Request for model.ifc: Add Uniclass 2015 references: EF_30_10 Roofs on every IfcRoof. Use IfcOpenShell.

First a look at what the model holds.

```python
import ifcopenshell

model = ifcopenshell.open("model.ifc")
print(model.schema)
print("classifications:", [c.Name for c in model.by_type("IfcClassification")])
for ifc_class in ("IfcDoor", "IfcRoof", "IfcStair", "IfcWall", "IfcWindow"):
    print(ifc_class, len(model.by_type(ifc_class)))
```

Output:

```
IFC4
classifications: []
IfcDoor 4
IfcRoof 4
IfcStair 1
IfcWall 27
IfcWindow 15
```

```python
import ifcopenshell
import ifcopenshell.api.classification

model = ifcopenshell.open("model.ifc")

system = ifcopenshell.api.classification.add_classification(model, classification="Uniclass 2015")

codes = {
    "IfcRoof": ("EF_30_10", "Roofs"),
}
for ifc_class, (code, name) in codes.items():
    products = model.by_type(ifc_class)
    ifcopenshell.api.classification.add_reference(
        model, products=products, classification=system, identification=code, name=name
    )
    print(code, len(products))

model.write("model-out.ifc")
```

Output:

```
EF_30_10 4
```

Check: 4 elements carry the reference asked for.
